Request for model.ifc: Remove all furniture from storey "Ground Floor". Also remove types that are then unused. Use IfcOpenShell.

First a look at what the model holds.

```python
import ifcopenshell
import ifcopenshell.util.element

model = ifcopenshell.open("model.ifc")
print(model.schema)
storey = next(s for s in model.by_type("IfcBuildingStorey") if s.Name == "Ground Floor")
furniture = [e for e in ifcopenshell.util.element.get_decomposition(storey) if e.is_a("IfcFurnishingElement")]
seen = {}
for e in furniture:
    element_type = ifcopenshell.util.element.get_type(e)
    name = element_type.Name if element_type not in (None, e) else None
    seen[name] = seen.get(name, 0) + 1
for name, count in sorted(seen.items(), key=str):
    print(count, "x", name)
```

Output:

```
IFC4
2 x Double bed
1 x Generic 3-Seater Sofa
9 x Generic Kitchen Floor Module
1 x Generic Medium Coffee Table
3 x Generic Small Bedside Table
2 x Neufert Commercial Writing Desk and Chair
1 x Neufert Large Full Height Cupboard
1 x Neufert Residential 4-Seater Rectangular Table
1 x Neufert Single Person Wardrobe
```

```python
import ifcopenshell
import ifcopenshell.api.root
import ifcopenshell.util.element

model = ifcopenshell.open("model.ifc")

storey = next(s for s in model.by_type("IfcBuildingStorey") if s.Name == "Ground Floor")
furniture = [e for e in ifcopenshell.util.element.get_decomposition(storey) if e.is_a("IfcFurnishingElement")]
types = {ifcopenshell.util.element.get_type(e) for e in furniture} - {None, *furniture}

for e in furniture:
    ifcopenshell.api.root.remove_product(model, product=e)
print(len(furniture), "removed")

unused = [t for t in types if not ifcopenshell.util.element.get_types(t)]
for t in unused:
    ifcopenshell.api.root.remove_product(model, product=t)
print(len(unused), "unused types removed")

model.write("model_v2.ifc")
```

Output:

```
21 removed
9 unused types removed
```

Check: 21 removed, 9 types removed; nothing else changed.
